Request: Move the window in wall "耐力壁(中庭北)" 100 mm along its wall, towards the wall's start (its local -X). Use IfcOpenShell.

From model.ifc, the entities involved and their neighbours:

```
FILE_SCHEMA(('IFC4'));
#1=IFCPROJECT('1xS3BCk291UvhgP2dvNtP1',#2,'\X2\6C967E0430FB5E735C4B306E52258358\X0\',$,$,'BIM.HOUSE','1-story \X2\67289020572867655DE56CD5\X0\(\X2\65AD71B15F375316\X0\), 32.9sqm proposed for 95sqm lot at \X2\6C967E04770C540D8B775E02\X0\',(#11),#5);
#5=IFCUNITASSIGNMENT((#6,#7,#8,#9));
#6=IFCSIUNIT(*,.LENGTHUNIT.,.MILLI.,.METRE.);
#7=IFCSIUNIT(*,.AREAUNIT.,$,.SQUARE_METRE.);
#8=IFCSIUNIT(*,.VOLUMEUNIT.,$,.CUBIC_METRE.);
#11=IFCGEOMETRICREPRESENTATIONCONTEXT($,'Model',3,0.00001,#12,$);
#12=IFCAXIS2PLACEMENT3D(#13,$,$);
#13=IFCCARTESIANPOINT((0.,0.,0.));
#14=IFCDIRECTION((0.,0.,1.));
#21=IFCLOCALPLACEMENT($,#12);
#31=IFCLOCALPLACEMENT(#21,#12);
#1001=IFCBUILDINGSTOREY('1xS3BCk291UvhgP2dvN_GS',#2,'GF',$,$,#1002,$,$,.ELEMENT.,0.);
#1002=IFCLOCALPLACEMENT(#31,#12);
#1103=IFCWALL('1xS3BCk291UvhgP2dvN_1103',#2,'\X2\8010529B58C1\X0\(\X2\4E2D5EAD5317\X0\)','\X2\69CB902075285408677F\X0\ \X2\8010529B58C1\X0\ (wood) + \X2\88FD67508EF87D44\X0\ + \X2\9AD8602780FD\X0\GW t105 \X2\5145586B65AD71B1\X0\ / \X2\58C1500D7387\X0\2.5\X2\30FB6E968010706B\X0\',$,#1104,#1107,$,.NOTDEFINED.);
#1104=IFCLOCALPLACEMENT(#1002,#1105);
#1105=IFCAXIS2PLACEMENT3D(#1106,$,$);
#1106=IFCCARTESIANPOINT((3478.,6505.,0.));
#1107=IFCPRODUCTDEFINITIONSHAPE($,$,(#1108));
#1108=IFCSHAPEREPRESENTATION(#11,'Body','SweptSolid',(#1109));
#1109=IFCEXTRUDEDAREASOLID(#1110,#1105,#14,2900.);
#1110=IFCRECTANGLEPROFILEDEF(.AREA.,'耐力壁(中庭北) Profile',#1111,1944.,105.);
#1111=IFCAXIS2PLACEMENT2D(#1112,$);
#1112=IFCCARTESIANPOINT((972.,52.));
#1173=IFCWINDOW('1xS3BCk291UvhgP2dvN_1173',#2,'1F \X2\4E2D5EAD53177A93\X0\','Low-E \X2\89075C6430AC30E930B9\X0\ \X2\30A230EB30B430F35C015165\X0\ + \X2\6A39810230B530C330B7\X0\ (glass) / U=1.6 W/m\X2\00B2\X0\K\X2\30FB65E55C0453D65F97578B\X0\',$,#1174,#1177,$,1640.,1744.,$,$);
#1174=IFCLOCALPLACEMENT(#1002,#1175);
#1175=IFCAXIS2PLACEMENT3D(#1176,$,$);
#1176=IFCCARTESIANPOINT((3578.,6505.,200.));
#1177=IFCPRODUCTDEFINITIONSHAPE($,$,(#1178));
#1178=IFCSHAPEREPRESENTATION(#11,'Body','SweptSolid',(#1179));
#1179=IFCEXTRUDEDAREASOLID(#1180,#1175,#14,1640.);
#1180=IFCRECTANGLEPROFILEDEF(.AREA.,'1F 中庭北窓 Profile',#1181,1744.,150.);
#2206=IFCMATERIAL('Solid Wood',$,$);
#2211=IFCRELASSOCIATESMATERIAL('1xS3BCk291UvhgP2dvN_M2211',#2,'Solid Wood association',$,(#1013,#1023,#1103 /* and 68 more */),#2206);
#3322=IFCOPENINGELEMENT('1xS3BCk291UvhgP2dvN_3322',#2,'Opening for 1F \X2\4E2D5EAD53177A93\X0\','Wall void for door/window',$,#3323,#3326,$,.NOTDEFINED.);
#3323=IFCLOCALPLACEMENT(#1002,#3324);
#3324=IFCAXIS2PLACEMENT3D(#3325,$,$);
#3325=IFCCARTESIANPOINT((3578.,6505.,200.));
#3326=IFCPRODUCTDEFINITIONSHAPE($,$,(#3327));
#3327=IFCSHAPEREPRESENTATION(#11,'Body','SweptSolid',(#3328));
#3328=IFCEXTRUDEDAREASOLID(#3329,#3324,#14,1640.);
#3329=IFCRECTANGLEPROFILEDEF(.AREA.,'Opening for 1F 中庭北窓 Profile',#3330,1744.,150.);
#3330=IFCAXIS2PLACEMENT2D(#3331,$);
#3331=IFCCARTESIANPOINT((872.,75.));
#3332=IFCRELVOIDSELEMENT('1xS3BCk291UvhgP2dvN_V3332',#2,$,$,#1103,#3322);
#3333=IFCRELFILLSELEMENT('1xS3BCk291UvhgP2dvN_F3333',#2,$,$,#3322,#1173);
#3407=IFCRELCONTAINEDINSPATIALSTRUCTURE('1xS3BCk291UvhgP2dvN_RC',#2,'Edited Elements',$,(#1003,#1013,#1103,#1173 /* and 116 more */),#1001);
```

```python
import ifcopenshell
import ifcopenshell.api.geometry
import ifcopenshell.util.placement
import ifcopenshell.util.unit

model = ifcopenshell.open("model.ifc")
unit_scale = ifcopenshell.util.unit.calculate_unit_scale(model)

window = model.by_guid("1xS3BCk291UvhgP2dvN_1173")
opening = window.FillsVoids[0].RelatingOpeningElement
wall = opening.VoidsElements[0].RelatingBuildingElement

wall_matrix = ifcopenshell.util.placement.get_local_placement(wall.ObjectPlacement)
shift = wall_matrix[:3, 0] * -0.1 / unit_scale
before = ifcopenshell.util.placement.get_local_placement(window.ObjectPlacement)[:3, 3].copy()

# The window is not placed relative to its opening, so move both.
for product in (opening, window):
    matrix = ifcopenshell.util.placement.get_local_placement(product.ObjectPlacement)
    matrix[:3, 3] += shift
    ifcopenshell.api.geometry.edit_object_placement(model, product=product, matrix=matrix, is_si=False)

after = ifcopenshell.util.placement.get_local_placement(window.ObjectPlacement)[:3, 3]
print("window moved by", (after - before).round(3) + 0.0)

model.write("model_edited.ifc")
```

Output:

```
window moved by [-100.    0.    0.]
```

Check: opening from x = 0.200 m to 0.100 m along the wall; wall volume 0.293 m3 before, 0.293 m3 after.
